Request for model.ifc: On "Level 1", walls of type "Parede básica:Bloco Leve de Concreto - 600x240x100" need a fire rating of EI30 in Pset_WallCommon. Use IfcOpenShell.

First a look at what the model holds.

```python
import ifcopenshell
import ifcopenshell.util.element

model = ifcopenshell.open("model.ifc")
print(model.schema)
storey = next(s for s in model.by_type("IfcBuildingStorey") if s.Name == "Level 1")
walls = [e for e in ifcopenshell.util.element.get_decomposition(storey) if e.is_a("IfcWall")]
seen = {}
for e in walls:
    element_type = ifcopenshell.util.element.get_type(e)
    key = (element_type.Name if element_type != e and element_type else None, ifcopenshell.util.element.get_pset(e, "Pset_WallCommon", "FireRating"))
    seen[key] = seen.get(key, 0) + 1
for (name, value), count in sorted(seen.items(), key=str):
    print(count, "x", name, "|", value)
```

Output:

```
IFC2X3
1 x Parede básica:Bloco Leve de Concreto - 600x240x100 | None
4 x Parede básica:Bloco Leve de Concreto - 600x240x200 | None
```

```python
import ifcopenshell
import ifcopenshell.api.pset
import ifcopenshell.util.element

model = ifcopenshell.open("model.ifc")

storey = next(s for s in model.by_type("IfcBuildingStorey") if s.Name == "Level 1")
walls = [e for e in ifcopenshell.util.element.get_decomposition(storey) if e.is_a("IfcWall")]

count = 0
for e in walls:
    element_type = ifcopenshell.util.element.get_type(e)
    if element_type in (None, e) or element_type.Name != "Parede básica:Bloco Leve de Concreto - 600x240x100":
        continue
    # add_pset returns the element's existing set when there is one.
    pset = ifcopenshell.api.pset.add_pset(model, product=e, name="Pset_WallCommon")
    ifcopenshell.api.pset.edit_pset(model, pset=pset, properties={"FireRating": "EI30"})
    count += 1

print(count, "walls updated")

model.write("model-out.ifc")
```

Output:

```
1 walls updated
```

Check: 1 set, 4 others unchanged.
